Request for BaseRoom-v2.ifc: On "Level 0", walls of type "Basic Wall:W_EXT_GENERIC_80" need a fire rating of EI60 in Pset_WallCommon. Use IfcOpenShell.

First a look at what the model holds.

```python
import ifcopenshell
import ifcopenshell.util.element

model = ifcopenshell.open("BaseRoom-v2.ifc")
print(model.schema)
storey = next(s for s in model.by_type("IfcBuildingStorey") if s.Name == "Level 0")
walls = [e for e in ifcopenshell.util.element.get_decomposition(storey) if e.is_a("IfcWall")]
seen = {}
for e in walls:
    element_type = ifcopenshell.util.element.get_type(e)
    key = (element_type.Name if element_type != e and element_type else None, ifcopenshell.util.element.get_pset(e, "Pset_WallCommon", "FireRating"))
    seen[key] = seen.get(key, 0) + 1
for (name, value), count in sorted(seen.items(), key=str):
    print(count, "x", name, "|", value)
```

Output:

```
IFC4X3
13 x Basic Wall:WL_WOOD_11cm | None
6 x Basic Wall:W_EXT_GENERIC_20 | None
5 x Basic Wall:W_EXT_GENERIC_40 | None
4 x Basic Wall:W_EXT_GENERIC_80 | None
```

```python
import ifcopenshell
import ifcopenshell.api.pset
import ifcopenshell.util.element

model = ifcopenshell.open("BaseRoom-v2.ifc")

storey = next(s for s in model.by_type("IfcBuildingStorey") if s.Name == "Level 0")
walls = [e for e in ifcopenshell.util.element.get_decomposition(storey) if e.is_a("IfcWall")]

count = 0
for e in walls:
    element_type = ifcopenshell.util.element.get_type(e)
    if element_type in (None, e) or element_type.Name != "Basic Wall:W_EXT_GENERIC_80":
        continue
    # add_pset returns the element's existing set when there is one.
    pset = ifcopenshell.api.pset.add_pset(model, product=e, name="Pset_WallCommon")
    ifcopenshell.api.pset.edit_pset(model, pset=pset, properties={"FireRating": "EI60"})
    count += 1

print(count, "walls updated")

model.write("BaseRoom-v2_edited.ifc")
```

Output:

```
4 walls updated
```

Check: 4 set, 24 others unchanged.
